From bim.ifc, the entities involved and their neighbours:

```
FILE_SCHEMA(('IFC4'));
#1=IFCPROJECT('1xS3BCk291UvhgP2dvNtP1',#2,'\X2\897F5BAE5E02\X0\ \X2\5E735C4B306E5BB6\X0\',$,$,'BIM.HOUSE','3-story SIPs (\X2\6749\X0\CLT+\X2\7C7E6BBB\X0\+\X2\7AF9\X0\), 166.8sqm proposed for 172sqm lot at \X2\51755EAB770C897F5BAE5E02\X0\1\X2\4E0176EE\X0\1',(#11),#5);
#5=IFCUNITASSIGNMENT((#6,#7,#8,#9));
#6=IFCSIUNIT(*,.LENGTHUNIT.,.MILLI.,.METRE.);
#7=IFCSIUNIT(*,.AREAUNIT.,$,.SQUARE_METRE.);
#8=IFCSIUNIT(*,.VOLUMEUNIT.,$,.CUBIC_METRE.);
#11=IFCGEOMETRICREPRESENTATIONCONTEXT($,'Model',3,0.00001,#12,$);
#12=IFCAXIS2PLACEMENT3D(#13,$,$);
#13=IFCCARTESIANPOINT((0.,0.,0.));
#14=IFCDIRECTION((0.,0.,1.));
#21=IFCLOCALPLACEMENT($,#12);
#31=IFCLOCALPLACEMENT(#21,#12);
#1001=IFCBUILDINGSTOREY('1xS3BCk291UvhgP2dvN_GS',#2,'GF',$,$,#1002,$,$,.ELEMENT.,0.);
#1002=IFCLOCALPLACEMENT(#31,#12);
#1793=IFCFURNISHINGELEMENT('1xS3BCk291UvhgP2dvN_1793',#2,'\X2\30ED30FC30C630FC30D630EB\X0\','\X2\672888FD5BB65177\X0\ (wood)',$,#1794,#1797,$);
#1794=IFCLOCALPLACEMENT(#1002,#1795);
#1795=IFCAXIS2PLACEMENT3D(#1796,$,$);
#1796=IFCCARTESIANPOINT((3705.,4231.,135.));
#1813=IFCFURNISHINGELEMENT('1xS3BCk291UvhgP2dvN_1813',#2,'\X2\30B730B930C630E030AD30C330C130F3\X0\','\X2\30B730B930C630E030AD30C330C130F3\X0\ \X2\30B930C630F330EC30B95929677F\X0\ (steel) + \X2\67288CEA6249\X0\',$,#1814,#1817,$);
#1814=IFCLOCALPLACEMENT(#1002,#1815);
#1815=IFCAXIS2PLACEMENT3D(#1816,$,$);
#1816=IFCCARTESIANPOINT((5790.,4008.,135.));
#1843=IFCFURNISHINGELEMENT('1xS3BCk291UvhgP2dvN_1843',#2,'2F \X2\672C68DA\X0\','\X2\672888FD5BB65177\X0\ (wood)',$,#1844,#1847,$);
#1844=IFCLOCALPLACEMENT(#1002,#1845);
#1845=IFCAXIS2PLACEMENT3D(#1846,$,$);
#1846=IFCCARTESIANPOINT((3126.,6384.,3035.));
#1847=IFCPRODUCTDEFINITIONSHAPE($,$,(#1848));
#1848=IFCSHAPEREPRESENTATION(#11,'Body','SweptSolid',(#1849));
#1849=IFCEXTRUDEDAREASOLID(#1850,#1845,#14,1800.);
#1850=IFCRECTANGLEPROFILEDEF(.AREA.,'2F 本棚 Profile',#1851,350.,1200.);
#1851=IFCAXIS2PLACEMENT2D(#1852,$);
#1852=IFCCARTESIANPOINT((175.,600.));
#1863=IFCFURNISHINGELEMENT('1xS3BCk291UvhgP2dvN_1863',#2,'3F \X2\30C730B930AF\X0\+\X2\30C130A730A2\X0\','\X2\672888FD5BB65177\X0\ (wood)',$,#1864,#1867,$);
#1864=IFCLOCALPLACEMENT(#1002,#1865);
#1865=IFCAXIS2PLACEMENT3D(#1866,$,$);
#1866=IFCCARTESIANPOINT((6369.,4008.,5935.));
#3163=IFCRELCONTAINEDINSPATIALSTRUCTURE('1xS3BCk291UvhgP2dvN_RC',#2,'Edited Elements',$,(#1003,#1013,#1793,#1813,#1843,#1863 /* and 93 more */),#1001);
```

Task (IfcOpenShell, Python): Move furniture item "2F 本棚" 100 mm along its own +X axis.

```python
import ifcopenshell
import ifcopenshell.api.geometry
import ifcopenshell.util.placement

model = ifcopenshell.open("bim.ifc")

item = model.by_id(1843)
matrix = ifcopenshell.util.placement.get_local_placement(item.ObjectPlacement)
matrix[:3, 3] += matrix[:3, 0] * 100.0
ifcopenshell.api.geometry.edit_object_placement(model, product=item, matrix=matrix, is_si=False)

print(ifcopenshell.util.placement.get_local_placement(item.ObjectPlacement).round(3) + 0.0)

model.write("bim-out.ifc")
```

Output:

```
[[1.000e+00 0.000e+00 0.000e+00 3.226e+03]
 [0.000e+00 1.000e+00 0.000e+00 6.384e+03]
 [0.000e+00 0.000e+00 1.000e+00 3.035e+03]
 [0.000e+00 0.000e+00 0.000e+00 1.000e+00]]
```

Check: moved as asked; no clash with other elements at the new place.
